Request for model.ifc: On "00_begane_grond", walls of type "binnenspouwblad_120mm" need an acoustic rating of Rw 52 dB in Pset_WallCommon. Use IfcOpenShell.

First a look at what the model holds.

```python
import ifcopenshell
import ifcopenshell.util.element

model = ifcopenshell.open("model.ifc")
print(model.schema)
storey = next(s for s in model.by_type("IfcBuildingStorey") if s.Name == "00_begane_grond")
walls = [e for e in ifcopenshell.util.element.get_decomposition(storey) if e.is_a("IfcWall")]
seen = {}
for e in walls:
    element_type = ifcopenshell.util.element.get_type(e)
    key = (element_type.Name if element_type != e and element_type else None, ifcopenshell.util.element.get_pset(e, "Pset_WallCommon", "AcousticRating"))
    seen[key] = seen.get(key, 0) + 1
for (name, value), count in sorted(seen.items(), key=str):
    print(count, "x", name, "|", value)
```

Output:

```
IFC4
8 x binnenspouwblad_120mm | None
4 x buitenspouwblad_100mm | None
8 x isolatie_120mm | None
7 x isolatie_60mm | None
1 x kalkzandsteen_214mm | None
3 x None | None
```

```python
import ifcopenshell
import ifcopenshell.api.pset
import ifcopenshell.util.element

model = ifcopenshell.open("model.ifc")

storey = next(s for s in model.by_type("IfcBuildingStorey") if s.Name == "00_begane_grond")
walls = [e for e in ifcopenshell.util.element.get_decomposition(storey) if e.is_a("IfcWall")]

count = 0
for e in walls:
    element_type = ifcopenshell.util.element.get_type(e)
    if element_type in (None, e) or element_type.Name != "binnenspouwblad_120mm":
        continue
    # add_pset returns the element's existing set when there is one.
    pset = ifcopenshell.api.pset.add_pset(model, product=e, name="Pset_WallCommon")
    ifcopenshell.api.pset.edit_pset(model, pset=pset, properties={"AcousticRating": "Rw 52 dB"})
    count += 1

print(count, "walls updated")

model.write("model_edited.ifc")
```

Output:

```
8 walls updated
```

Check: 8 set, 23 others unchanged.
